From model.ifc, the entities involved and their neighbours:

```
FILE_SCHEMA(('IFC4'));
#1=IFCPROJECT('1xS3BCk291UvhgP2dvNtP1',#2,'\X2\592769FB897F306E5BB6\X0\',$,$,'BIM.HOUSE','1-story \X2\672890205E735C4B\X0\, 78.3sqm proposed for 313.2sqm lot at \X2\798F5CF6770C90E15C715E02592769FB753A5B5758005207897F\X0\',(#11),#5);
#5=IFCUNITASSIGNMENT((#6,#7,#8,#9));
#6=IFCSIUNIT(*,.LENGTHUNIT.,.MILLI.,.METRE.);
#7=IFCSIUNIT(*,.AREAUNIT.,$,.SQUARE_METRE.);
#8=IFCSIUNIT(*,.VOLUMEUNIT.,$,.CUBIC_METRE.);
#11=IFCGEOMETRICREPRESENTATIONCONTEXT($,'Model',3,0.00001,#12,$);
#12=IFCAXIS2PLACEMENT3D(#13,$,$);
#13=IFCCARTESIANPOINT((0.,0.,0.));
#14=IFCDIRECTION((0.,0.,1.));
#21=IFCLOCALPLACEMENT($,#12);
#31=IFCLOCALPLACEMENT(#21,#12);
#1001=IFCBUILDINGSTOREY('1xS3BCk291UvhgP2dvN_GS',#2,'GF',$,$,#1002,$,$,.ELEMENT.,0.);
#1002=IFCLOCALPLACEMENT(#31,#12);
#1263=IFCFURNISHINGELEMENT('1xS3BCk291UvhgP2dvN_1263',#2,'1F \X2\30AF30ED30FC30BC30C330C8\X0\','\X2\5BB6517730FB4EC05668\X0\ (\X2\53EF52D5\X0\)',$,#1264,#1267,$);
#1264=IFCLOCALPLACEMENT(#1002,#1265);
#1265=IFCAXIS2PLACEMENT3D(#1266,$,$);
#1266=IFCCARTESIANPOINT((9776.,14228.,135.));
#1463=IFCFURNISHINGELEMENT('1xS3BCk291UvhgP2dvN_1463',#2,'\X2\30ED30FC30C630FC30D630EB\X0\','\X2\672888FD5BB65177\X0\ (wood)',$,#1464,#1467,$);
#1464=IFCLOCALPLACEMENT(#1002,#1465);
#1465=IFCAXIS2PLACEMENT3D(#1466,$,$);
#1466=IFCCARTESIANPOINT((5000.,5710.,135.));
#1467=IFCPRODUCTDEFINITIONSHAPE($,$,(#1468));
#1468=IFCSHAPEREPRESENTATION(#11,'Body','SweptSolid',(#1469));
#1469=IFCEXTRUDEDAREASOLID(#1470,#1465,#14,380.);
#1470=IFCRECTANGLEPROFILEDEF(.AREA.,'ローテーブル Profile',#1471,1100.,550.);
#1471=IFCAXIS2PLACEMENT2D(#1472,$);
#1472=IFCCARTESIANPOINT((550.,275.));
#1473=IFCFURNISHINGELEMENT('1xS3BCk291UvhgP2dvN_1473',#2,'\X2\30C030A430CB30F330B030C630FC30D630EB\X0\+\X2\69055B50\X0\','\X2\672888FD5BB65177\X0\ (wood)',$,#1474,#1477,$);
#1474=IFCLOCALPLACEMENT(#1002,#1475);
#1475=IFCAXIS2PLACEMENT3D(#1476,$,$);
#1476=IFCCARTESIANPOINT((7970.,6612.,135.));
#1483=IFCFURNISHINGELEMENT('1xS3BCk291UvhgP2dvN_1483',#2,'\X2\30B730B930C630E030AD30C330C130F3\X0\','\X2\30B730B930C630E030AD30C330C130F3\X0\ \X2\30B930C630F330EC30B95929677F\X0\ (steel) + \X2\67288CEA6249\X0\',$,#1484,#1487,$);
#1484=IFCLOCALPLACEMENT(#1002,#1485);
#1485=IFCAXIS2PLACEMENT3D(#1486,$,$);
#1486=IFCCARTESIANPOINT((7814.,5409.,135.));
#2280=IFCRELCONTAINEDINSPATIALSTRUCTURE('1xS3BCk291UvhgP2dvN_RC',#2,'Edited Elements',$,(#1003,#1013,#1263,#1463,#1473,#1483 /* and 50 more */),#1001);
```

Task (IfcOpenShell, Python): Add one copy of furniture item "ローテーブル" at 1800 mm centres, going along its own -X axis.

```python
import ifcopenshell
import ifcopenshell.api.geometry
import ifcopenshell.api.root
import ifcopenshell.util.element
import ifcopenshell.util.placement

model = ifcopenshell.open("model.ifc")


def reuse_history(source, copy):
    """copy_class also copies each property set's owner history, people and application; keep the originals."""
    for rel in copy.IsDefinedBy:
        if rel.is_a("IfcRelDefinesByProperties") and (history := rel.RelatingPropertyDefinition.OwnerHistory):
            rel.RelatingPropertyDefinition.OwnerHistory = source.OwnerHistory
            ifcopenshell.util.element.remove_deep2(model, history)


source = model.by_guid("1xS3BCk291UvhgP2dvN_1463")
base = ifcopenshell.util.placement.get_local_placement(source.ObjectPlacement)
step = -base[:3, 0] * 1800.0

for i in range(1, 2):
    copy = ifcopenshell.api.root.copy_class(model, product=source)
    copy.Representation = ifcopenshell.util.element.copy_deep(
        model, source.Representation, exclude=["IfcGeometricRepresentationContext", "IfcRepresentationMap"]
    )
    reuse_history(source, copy)
    matrix = base.copy()
    matrix[:3, 3] += i * step
    print("added at", matrix[:3, 3].round(3) + 0.0)
    ifcopenshell.api.geometry.edit_object_placement(model, product=copy, matrix=matrix, is_si=False)

model.write("model-out.ifc")
```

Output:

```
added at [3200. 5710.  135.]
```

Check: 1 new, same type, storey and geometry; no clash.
